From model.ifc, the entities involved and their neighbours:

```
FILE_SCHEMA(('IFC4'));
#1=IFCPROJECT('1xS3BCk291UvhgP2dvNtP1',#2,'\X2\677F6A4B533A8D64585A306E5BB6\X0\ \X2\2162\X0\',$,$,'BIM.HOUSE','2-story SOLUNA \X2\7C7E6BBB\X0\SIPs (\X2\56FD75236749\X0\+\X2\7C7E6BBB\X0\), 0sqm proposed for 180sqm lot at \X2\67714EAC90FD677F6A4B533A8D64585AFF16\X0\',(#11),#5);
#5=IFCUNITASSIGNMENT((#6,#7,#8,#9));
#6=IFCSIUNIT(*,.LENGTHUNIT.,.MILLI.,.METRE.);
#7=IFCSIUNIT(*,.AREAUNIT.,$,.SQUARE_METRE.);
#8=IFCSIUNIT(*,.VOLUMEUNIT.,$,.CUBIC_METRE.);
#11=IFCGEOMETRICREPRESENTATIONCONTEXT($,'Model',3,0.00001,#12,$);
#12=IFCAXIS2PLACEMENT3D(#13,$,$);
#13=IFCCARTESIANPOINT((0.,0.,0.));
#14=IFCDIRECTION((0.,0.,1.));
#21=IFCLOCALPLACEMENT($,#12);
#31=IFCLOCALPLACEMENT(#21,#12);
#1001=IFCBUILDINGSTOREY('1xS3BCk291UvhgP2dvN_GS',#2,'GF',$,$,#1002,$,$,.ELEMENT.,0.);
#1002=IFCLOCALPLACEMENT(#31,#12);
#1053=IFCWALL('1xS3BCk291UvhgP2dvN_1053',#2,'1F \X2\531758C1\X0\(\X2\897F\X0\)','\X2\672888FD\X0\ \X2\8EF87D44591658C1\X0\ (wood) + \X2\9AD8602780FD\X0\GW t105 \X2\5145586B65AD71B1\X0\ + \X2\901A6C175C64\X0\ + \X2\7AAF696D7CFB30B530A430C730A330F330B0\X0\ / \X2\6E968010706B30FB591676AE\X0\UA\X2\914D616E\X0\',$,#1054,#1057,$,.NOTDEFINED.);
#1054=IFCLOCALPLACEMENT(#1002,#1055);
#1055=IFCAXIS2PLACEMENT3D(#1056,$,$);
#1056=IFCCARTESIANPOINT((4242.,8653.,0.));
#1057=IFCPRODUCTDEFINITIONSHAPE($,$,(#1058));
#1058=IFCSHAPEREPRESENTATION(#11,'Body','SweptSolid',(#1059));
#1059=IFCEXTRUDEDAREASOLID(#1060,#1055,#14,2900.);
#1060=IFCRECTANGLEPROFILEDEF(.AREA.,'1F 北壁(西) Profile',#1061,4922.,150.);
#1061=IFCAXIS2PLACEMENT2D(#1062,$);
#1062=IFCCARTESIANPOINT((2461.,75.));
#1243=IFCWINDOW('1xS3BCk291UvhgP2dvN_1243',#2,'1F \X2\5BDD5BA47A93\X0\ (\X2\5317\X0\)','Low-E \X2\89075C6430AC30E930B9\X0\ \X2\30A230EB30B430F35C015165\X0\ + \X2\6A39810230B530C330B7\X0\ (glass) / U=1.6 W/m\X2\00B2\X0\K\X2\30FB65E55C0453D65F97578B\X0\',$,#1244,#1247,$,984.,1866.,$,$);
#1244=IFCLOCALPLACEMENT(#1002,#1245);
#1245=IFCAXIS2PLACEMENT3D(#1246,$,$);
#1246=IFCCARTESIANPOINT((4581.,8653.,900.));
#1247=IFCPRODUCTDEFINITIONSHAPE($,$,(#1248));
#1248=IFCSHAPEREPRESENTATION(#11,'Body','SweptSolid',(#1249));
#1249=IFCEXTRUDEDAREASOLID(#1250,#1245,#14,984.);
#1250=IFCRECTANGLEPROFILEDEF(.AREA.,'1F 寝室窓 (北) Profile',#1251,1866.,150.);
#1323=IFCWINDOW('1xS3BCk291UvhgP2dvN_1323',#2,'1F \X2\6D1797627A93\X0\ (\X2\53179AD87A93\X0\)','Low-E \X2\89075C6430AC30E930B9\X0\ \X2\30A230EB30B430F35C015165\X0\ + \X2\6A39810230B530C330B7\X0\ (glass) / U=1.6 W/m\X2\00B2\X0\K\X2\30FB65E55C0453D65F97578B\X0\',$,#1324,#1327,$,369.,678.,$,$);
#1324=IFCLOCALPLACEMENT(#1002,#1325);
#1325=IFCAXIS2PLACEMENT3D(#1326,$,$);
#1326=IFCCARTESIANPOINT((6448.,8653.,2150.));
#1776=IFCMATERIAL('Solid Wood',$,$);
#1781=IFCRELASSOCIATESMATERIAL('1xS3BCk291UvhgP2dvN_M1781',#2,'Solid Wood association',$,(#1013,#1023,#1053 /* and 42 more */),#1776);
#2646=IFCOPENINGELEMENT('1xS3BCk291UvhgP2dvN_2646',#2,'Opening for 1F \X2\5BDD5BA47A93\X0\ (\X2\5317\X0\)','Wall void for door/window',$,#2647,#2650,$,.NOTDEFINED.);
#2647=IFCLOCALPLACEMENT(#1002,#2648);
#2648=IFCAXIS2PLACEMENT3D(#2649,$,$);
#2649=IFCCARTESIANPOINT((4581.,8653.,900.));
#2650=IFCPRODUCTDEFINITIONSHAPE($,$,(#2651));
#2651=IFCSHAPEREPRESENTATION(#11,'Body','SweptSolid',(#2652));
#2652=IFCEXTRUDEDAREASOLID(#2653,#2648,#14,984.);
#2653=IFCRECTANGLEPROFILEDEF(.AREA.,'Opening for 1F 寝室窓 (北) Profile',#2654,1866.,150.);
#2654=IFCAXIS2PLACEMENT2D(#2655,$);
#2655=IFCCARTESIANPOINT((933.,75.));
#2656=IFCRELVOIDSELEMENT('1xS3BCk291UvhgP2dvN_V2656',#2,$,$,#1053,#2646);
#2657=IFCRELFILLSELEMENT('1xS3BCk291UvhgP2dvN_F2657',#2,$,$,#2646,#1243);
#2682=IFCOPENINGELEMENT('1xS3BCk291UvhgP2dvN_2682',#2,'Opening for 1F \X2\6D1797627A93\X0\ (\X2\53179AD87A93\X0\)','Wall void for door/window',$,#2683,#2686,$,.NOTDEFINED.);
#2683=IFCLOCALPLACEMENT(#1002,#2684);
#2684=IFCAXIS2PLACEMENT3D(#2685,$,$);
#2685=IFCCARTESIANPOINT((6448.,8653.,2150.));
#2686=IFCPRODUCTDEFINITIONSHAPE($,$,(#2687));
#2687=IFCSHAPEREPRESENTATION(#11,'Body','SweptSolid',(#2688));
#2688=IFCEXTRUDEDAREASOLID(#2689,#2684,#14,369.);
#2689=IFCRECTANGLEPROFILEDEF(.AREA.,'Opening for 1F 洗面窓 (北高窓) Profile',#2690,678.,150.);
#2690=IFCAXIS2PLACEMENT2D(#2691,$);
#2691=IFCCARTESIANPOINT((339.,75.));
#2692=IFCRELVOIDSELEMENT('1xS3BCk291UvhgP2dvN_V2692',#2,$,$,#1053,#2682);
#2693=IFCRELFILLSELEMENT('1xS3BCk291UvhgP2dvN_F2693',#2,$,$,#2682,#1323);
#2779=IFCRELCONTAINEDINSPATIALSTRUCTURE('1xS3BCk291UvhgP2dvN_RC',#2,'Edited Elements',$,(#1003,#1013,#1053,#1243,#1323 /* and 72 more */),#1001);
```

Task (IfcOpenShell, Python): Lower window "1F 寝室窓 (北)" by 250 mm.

```python
import numpy as np
import ifcopenshell
import ifcopenshell.api.geometry
import ifcopenshell.util.placement
import ifcopenshell.util.unit

model = ifcopenshell.open("model.ifc")
unit_scale = ifcopenshell.util.unit.calculate_unit_scale(model)

window = model.by_guid("1xS3BCk291UvhgP2dvN_1243")
opening = window.FillsVoids[0].RelatingOpeningElement
dz = -0.25 / unit_scale

shift = np.array([0.0, 0.0, dz])
# The window is not placed relative to its opening, so move both.
for product in (opening, window):
    matrix = ifcopenshell.util.placement.get_local_placement(product.ObjectPlacement)
    matrix[:3, 3] += shift
    ifcopenshell.api.geometry.edit_object_placement(model, product=product, matrix=matrix, is_si=False)

print(f"moved by {dz * unit_scale:+.3f} m")

model.write("model-out.ifc")
```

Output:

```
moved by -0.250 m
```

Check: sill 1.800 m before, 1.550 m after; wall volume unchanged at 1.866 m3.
